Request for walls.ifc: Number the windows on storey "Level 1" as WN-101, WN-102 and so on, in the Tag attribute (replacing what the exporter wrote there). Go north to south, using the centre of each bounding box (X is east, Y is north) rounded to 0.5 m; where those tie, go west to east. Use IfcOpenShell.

First a look at what the model holds.

```python
import ifcopenshell
import ifcopenshell.util.element
import ifcopenshell.util.placement

model = ifcopenshell.open("walls.ifc")
print(model.schema)
storey = next(s for s in model.by_type("IfcBuildingStorey") if s.Name == "Level 1")
windows = [e for e in ifcopenshell.util.element.get_decomposition(storey) if e.is_a("IfcWindow")]
for e in sorted(windows, key=lambda e: e.id()):
    origin = ifcopenshell.util.placement.get_local_placement(e.ObjectPlacement)[:3, 3]
    print(e.id(), e.Tag, e.Name, origin.round(2) + 0.0, sep=" | ")
```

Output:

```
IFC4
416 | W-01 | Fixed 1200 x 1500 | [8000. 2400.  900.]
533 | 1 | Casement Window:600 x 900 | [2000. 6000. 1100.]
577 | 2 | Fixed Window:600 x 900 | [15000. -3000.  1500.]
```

```python
import ifcopenshell
import ifcopenshell.geom
import ifcopenshell.util.element
import ifcopenshell.util.shape

model = ifcopenshell.open("walls.ifc")
settings = ifcopenshell.geom.settings()
settings.set("use-world-coords", True)


def centre(element):
    shape = ifcopenshell.geom.create_shape(settings, element)
    return ifcopenshell.util.shape.get_bbox_centroid(shape.geometry)


storey = next(s for s in model.by_type("IfcBuildingStorey") if s.Name == "Level 1")
windows = [e for e in ifcopenshell.util.element.get_decomposition(storey) if e.is_a("IfcWindow")]

# Insertion points can sit at a corner or the storey origin, so sort by the geometry (in metres).
centres = {e: centre(e) for e in windows}
windows.sort(key=lambda e: (-round(centres[e][1] / 0.5), centres[e][0]))

for i, e in enumerate(windows, start=1):
    number = f"WN-1{i:02d}"
    e.Tag = number
    print(e.id(), number)

model.write("walls_rev.ifc")
```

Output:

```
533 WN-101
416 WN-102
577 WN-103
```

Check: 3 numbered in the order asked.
